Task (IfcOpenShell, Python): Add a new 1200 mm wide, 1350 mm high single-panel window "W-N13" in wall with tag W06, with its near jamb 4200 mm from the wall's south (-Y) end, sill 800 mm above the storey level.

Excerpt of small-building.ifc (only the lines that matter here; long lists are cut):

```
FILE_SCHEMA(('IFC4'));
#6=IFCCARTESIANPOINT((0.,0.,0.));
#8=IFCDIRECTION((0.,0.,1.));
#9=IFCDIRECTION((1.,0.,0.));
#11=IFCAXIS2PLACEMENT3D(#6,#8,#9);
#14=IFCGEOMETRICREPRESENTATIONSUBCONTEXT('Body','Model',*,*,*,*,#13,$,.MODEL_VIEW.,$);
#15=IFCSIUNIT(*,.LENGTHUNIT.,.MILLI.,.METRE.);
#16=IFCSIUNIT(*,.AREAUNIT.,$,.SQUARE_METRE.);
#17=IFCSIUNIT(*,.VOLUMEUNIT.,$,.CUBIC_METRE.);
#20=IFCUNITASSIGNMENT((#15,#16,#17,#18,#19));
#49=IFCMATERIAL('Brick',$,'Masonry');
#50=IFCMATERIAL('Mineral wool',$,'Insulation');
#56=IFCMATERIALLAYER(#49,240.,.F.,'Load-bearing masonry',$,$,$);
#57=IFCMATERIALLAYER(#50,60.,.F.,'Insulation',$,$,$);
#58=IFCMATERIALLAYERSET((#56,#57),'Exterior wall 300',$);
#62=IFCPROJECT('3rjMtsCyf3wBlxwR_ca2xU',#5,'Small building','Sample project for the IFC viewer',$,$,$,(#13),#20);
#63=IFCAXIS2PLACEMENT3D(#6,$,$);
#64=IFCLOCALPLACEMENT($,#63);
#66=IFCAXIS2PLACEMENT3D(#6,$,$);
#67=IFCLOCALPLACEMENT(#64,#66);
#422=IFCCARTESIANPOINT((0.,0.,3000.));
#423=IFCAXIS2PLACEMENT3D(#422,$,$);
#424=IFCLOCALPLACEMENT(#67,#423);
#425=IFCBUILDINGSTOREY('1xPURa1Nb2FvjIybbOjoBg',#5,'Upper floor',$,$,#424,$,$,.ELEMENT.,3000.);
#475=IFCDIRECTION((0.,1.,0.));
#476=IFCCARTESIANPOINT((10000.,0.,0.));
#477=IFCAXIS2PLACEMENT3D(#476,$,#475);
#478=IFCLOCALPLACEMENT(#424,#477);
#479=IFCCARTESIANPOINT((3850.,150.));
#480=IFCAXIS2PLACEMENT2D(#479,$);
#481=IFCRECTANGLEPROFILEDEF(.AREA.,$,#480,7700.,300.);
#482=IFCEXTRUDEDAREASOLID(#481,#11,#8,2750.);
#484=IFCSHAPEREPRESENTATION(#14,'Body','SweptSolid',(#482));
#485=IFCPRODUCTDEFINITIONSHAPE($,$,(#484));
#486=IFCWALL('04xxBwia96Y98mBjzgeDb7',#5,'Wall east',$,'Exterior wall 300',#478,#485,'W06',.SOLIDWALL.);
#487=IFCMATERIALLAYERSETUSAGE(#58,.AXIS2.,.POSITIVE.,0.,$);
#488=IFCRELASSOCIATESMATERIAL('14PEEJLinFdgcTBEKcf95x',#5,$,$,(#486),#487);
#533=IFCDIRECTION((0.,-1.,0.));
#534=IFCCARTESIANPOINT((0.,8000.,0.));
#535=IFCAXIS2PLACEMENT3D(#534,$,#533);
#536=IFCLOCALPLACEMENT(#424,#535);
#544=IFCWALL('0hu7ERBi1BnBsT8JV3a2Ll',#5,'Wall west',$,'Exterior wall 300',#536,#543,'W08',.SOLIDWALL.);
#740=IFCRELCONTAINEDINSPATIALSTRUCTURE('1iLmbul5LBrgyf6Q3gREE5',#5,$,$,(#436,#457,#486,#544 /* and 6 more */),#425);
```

```python
import numpy as np
import ifcopenshell
import ifcopenshell.api.feature
import ifcopenshell.api.geometry
import ifcopenshell.api.root
import ifcopenshell.api.spatial
import ifcopenshell.geom
import ifcopenshell.util.element
import ifcopenshell.util.placement
import ifcopenshell.util.representation
import ifcopenshell.util.shape
import ifcopenshell.util.unit

model = ifcopenshell.open("small-building.ifc")
unit_scale = ifcopenshell.util.unit.calculate_unit_scale(model)
settings = ifcopenshell.geom.settings()


def volume(element):
    """Net volume in cubic metres, openings subtracted."""
    shape = ifcopenshell.geom.create_shape(settings, element)
    return ifcopenshell.util.shape.get_volume(shape.geometry)


wall = model.by_guid("04xxBwia96Y98mBjzgeDb7")
storey = ifcopenshell.util.element.get_container(wall, ifc_class="IfcBuildingStorey")
context = ifcopenshell.util.representation.get_context(model, "Model", "Body", "MODEL_VIEW")
before = volume(wall)

width, height, from_end, sill = 1.2, 1.35, 4.2, 0.8  # metres

# The wall runs along its own X axis, and the end named is its -X end.
wall_shape = ifcopenshell.geom.create_shape(settings, wall)
x, y, z = ifcopenshell.util.shape.get_vertices(wall_shape.geometry).T
start = x.min() + from_end
face, thickness = float(y.min()), float(y.max() - y.min())
wall_matrix = ifcopenshell.util.placement.get_local_placement(wall.ObjectPlacement)
level = ifcopenshell.util.placement.get_local_placement(storey.ObjectPlacement)[2, 3]


def in_wall(x, y):
    """Placement at x, y metres in the wall's axes, at sill height."""
    matrix = wall_matrix.copy()
    matrix[:, 3] = wall_matrix @ np.array([x / unit_scale, y / unit_scale, 0.0, 1.0])
    matrix[2, 3] = level + sill / unit_scale
    return matrix


# Opening: a box that overshoots both wall faces by 50 mm.
opening = ifcopenshell.api.root.create_entity(model, ifc_class="IfcOpeningElement", predefined_type="OPENING")
box = ifcopenshell.api.geometry.add_wall_representation(
    model, context=context, length=width, height=height, thickness=thickness + 0.1
)
ifcopenshell.api.geometry.assign_representation(model, product=opening, representation=box)
ifcopenshell.api.geometry.edit_object_placement(model, product=opening, matrix=in_wall(start, face - 0.05), is_si=False)
ifcopenshell.api.feature.add_feature(model, feature=opening, element=wall)

window = ifcopenshell.api.root.create_entity(model, ifc_class="IfcWindow", name="W-N13", predefined_type="WINDOW")
window.OverallWidth, window.OverallHeight = width / unit_scale, height / unit_scale
window.PartitioningType = "SINGLE_PANEL"
body = ifcopenshell.api.geometry.add_window_representation(
    model,
    context=context,
    overall_width=window.OverallWidth,
    overall_height=window.OverallHeight,
    partition_type="SINGLE_PANEL",
)
ifcopenshell.api.geometry.assign_representation(model, product=window, representation=body)
ifcopenshell.api.spatial.assign_container(model, products=[window], relating_structure=storey)
ifcopenshell.api.feature.add_filling(model, opening=opening, element=window)

# Centre the window in the wall's thickness.
ifcopenshell.api.geometry.edit_object_placement(model, product=window, matrix=in_wall(start, face), is_si=False)
window_shape = ifcopenshell.geom.create_shape(settings, window)
depth = ifcopenshell.util.shape.get_vertices(window_shape.geometry)[:, 1]
offset = face + thickness / 2 - (depth.min() + depth.max()) / 2
ifcopenshell.api.geometry.edit_object_placement(model, product=window, matrix=in_wall(start, offset), is_si=False)

after = volume(wall)

print(f"wall volume {before:.3f} -> {after:.3f} m3")

model.write("small-building_rev.ifc")
```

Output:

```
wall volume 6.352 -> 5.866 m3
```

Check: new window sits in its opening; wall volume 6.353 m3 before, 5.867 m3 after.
